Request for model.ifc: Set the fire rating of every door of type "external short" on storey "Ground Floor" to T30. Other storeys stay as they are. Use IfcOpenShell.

First a look at what the model holds.

```python
import ifcopenshell
import ifcopenshell.util.element

model = ifcopenshell.open("model.ifc")
print(model.schema)
storey = next(s for s in model.by_type("IfcBuildingStorey") if s.Name == "Ground Floor")
doors = [e for e in ifcopenshell.util.element.get_decomposition(storey) if e.is_a("IfcDoor")]
seen = {}
for e in doors:
    element_type = ifcopenshell.util.element.get_type(e)
    key = (element_type.Name if element_type != e and element_type else None, ifcopenshell.util.element.get_pset(e, "Pset_DoorCommon", "FireRating"))
    seen[key] = seen.get(key, 0) + 1
for (name, value), count in sorted(seen.items(), key=str):
    print(count, "x", name, "|", value)
```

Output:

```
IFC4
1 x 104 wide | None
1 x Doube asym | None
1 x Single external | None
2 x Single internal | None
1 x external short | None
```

```python
import ifcopenshell
import ifcopenshell.api.pset
import ifcopenshell.util.element

model = ifcopenshell.open("model.ifc")

storey = next(s for s in model.by_type("IfcBuildingStorey") if s.Name == "Ground Floor")
doors = [e for e in ifcopenshell.util.element.get_decomposition(storey) if e.is_a("IfcDoor")]

count = 0
for e in doors:
    element_type = ifcopenshell.util.element.get_type(e)
    if element_type in (None, e) or element_type.Name != "external short":
        continue
    # add_pset returns the element's existing set when there is one.
    pset = ifcopenshell.api.pset.add_pset(model, product=e, name="Pset_DoorCommon")
    ifcopenshell.api.pset.edit_pset(model, pset=pset, properties={"FireRating": "T30"})
    count += 1

print(count, "doors updated")

model.write("model_updated.ifc")
```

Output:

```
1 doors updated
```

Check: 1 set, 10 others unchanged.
